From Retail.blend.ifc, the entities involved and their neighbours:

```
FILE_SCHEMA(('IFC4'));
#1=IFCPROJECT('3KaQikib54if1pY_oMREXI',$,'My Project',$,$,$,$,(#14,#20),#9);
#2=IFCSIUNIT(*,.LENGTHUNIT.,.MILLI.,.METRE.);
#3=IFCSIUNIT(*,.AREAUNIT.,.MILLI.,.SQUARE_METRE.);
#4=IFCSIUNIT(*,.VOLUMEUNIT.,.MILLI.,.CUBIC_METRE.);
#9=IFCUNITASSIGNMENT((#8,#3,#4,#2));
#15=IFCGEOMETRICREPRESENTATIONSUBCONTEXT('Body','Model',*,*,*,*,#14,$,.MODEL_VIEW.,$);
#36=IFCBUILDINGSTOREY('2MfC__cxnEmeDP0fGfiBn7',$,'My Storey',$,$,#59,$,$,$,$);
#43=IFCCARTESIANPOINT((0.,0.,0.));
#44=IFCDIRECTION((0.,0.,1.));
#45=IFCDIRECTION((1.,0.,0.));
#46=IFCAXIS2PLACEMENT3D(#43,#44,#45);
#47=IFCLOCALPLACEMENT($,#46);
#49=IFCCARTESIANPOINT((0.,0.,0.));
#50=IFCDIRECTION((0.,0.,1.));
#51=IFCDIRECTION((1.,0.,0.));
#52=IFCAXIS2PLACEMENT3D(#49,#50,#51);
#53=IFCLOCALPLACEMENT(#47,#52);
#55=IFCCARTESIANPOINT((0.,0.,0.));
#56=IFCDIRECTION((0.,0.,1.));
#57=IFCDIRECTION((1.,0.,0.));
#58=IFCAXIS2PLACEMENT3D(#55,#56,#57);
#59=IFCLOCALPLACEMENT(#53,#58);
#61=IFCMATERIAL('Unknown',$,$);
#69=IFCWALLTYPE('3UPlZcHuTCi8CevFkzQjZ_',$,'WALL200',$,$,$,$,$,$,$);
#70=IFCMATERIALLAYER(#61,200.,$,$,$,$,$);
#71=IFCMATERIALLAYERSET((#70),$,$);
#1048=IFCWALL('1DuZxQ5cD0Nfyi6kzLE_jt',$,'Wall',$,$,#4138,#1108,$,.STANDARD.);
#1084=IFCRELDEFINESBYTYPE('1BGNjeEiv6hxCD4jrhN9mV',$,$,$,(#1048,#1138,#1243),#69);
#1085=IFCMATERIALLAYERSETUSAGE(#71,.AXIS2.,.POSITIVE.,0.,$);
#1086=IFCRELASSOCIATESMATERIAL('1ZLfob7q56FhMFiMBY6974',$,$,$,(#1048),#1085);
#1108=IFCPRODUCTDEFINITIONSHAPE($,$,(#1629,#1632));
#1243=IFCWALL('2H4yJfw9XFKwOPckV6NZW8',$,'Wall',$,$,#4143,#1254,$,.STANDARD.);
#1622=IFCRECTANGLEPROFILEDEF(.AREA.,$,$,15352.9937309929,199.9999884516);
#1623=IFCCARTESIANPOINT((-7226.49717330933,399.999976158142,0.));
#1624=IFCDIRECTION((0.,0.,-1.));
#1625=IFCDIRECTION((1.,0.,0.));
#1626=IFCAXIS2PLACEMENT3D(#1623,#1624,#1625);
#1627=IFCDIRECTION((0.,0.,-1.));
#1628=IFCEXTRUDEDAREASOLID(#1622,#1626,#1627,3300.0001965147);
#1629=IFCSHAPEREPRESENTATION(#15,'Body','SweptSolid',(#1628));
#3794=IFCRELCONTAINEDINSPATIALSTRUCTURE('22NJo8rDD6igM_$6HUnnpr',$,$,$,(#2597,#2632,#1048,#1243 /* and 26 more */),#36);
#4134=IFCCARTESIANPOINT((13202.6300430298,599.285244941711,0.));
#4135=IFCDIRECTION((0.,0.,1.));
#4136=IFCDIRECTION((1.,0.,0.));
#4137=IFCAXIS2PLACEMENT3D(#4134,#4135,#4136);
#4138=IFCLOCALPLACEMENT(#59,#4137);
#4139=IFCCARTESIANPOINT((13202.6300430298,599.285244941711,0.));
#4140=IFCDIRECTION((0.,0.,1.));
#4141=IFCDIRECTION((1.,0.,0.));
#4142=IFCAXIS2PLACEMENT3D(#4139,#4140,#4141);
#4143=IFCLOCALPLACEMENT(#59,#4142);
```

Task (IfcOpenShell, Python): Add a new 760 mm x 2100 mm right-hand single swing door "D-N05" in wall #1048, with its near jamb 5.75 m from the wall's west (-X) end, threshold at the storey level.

```python
import numpy as np
import ifcopenshell
import ifcopenshell.api.feature
import ifcopenshell.api.geometry
import ifcopenshell.api.root
import ifcopenshell.api.spatial
import ifcopenshell.geom
import ifcopenshell.util.element
import ifcopenshell.util.placement
import ifcopenshell.util.representation
import ifcopenshell.util.shape
import ifcopenshell.util.unit

model = ifcopenshell.open("Retail.blend.ifc")
unit_scale = ifcopenshell.util.unit.calculate_unit_scale(model)
settings = ifcopenshell.geom.settings()


def volume(element):
    """Net volume in cubic metres, openings subtracted."""
    shape = ifcopenshell.geom.create_shape(settings, element)
    return ifcopenshell.util.shape.get_volume(shape.geometry)


wall = model.by_guid("1DuZxQ5cD0Nfyi6kzLE_jt")
storey = ifcopenshell.util.element.get_container(wall, ifc_class="IfcBuildingStorey")
context = ifcopenshell.util.representation.get_context(model, "Model", "Body", "MODEL_VIEW")
before = volume(wall)

width, height, from_end, sill = 0.76, 2.1, 5.75, 0.0  # metres

# The wall runs along its own X axis, and the end named is its -X end.
wall_shape = ifcopenshell.geom.create_shape(settings, wall)
x, y, z = ifcopenshell.util.shape.get_vertices(wall_shape.geometry).T
start = x.min() + from_end
face, thickness = float(y.min()), float(y.max() - y.min())
wall_matrix = ifcopenshell.util.placement.get_local_placement(wall.ObjectPlacement)
level = ifcopenshell.util.placement.get_local_placement(storey.ObjectPlacement)[2, 3]


def in_wall(x, y):
    """Placement at x, y metres in the wall's axes, at sill height."""
    matrix = wall_matrix.copy()
    matrix[:, 3] = wall_matrix @ np.array([x / unit_scale, y / unit_scale, 0.0, 1.0])
    matrix[2, 3] = level + sill / unit_scale
    return matrix


# Opening: a box that overshoots both wall faces by 50 mm.
opening = ifcopenshell.api.root.create_entity(model, ifc_class="IfcOpeningElement", predefined_type="OPENING")
box = ifcopenshell.api.geometry.add_wall_representation(
    model, context=context, length=width, height=height, thickness=thickness + 0.1
)
ifcopenshell.api.geometry.assign_representation(model, product=opening, representation=box)
ifcopenshell.api.geometry.edit_object_placement(model, product=opening, matrix=in_wall(start, face - 0.05), is_si=False)
ifcopenshell.api.feature.add_feature(model, feature=opening, element=wall)

door = ifcopenshell.api.root.create_entity(model, ifc_class="IfcDoor", name="D-N05", predefined_type="DOOR")
door.OverallWidth, door.OverallHeight = width / unit_scale, height / unit_scale
door.OperationType = "SINGLE_SWING_RIGHT"
body = ifcopenshell.api.geometry.add_door_representation(
    model,
    context=context,
    overall_width=door.OverallWidth,
    overall_height=door.OverallHeight,
    operation_type="SINGLE_SWING_RIGHT",
    lining_properties={"LiningDepth": thickness / unit_scale, "ThresholdDepth": thickness / unit_scale},
)
ifcopenshell.api.geometry.assign_representation(model, product=door, representation=body)
ifcopenshell.api.spatial.assign_container(model, products=[door], relating_structure=storey)
ifcopenshell.api.feature.add_filling(model, opening=opening, element=door)

# The lining spans the wall, so the door starts at the wall face.
ifcopenshell.api.geometry.edit_object_placement(model, product=door, matrix=in_wall(start, face), is_si=False)

after = volume(wall)

print(f"wall volume {before:.3f} -> {after:.3f} m3")

model.write("Retail.blend_edited.ifc")
```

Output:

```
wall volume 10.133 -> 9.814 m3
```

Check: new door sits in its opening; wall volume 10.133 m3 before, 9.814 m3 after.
